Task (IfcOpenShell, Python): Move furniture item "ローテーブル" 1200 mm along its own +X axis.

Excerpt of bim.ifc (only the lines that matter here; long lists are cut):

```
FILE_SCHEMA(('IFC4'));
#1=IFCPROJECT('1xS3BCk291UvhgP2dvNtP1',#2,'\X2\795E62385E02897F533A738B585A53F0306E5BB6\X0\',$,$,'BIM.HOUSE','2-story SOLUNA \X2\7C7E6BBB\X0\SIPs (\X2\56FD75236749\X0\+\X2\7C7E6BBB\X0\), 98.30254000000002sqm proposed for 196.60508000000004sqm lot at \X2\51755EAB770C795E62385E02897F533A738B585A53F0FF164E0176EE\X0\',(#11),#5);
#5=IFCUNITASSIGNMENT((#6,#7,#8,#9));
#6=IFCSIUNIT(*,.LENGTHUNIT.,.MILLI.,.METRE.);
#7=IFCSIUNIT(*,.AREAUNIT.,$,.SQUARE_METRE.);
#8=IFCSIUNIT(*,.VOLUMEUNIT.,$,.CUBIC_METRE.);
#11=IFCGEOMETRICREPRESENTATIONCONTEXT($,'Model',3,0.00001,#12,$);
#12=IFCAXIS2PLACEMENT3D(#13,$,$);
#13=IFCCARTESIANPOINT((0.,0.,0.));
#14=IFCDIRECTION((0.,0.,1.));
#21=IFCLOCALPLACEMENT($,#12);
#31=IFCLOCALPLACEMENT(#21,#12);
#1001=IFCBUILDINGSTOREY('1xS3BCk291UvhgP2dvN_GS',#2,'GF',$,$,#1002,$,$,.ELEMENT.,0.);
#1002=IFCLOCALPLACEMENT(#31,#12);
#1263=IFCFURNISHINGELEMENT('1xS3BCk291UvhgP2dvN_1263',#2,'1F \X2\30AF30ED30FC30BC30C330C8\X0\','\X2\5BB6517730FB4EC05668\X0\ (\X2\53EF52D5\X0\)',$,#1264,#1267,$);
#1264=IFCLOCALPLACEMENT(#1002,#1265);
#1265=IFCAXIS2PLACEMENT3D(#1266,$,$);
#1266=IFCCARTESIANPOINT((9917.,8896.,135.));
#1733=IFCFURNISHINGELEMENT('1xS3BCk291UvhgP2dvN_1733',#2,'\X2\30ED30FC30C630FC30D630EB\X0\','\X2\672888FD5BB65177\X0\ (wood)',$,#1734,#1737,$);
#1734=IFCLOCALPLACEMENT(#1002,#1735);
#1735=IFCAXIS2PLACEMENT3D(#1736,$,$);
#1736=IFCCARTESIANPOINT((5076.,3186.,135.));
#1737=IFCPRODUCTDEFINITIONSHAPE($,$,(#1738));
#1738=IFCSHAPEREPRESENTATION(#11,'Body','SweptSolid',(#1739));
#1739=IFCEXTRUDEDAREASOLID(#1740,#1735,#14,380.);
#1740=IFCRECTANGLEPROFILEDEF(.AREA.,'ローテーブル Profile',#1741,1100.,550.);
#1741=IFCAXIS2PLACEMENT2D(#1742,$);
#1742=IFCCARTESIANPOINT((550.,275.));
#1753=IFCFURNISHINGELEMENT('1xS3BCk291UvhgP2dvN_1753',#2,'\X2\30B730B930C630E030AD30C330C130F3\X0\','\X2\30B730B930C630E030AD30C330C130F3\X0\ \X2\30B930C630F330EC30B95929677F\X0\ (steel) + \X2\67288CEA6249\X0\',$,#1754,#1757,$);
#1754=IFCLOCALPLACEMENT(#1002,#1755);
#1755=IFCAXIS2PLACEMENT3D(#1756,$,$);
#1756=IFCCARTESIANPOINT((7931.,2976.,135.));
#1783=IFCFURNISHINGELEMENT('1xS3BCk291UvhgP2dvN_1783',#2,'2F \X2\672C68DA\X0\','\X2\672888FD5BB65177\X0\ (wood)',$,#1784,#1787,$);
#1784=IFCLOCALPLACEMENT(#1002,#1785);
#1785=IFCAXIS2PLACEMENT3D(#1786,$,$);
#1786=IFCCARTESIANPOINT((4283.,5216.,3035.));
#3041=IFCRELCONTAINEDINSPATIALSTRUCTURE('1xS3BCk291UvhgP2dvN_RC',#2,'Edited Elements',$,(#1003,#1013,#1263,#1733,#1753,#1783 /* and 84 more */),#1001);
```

```python
import ifcopenshell
import ifcopenshell.api.geometry
import ifcopenshell.util.placement

model = ifcopenshell.open("bim.ifc")

item = model.by_guid("1xS3BCk291UvhgP2dvN_1733")
matrix = ifcopenshell.util.placement.get_local_placement(item.ObjectPlacement)
matrix[:3, 3] += matrix[:3, 0] * 1200.0
ifcopenshell.api.geometry.edit_object_placement(model, product=item, matrix=matrix, is_si=False)

print(ifcopenshell.util.placement.get_local_placement(item.ObjectPlacement).round(3) + 0.0)

model.write("bim-out.ifc")
```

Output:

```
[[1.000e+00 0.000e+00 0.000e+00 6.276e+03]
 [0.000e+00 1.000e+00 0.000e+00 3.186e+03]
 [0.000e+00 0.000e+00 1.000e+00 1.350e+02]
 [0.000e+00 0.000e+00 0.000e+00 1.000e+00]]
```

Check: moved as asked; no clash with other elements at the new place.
